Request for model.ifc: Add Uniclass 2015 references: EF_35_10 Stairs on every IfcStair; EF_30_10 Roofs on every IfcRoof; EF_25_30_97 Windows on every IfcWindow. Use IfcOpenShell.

First a look at what the model holds.

```python
import ifcopenshell

model = ifcopenshell.open("model.ifc")
print(model.schema)
print("classifications:", [c.Name for c in model.by_type("IfcClassification")])
for ifc_class in ("IfcDoor", "IfcRoof", "IfcStair", "IfcWall", "IfcWindow"):
    print(ifc_class, len(model.by_type(ifc_class)))
```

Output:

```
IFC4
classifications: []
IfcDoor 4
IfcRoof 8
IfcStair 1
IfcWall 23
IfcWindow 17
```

```python
import ifcopenshell
import ifcopenshell.api.classification

model = ifcopenshell.open("model.ifc")

system = ifcopenshell.api.classification.add_classification(model, classification="Uniclass 2015")

codes = {
    "IfcStair": ("EF_35_10", "Stairs"),
    "IfcRoof": ("EF_30_10", "Roofs"),
    "IfcWindow": ("EF_25_30_97", "Windows"),
}
for ifc_class, (code, name) in codes.items():
    products = model.by_type(ifc_class)
    ifcopenshell.api.classification.add_reference(
        model, products=products, classification=system, identification=code, name=name
    )
    print(code, len(products))

model.write("model_rev.ifc")
```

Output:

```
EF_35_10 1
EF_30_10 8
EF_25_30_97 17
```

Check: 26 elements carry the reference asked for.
